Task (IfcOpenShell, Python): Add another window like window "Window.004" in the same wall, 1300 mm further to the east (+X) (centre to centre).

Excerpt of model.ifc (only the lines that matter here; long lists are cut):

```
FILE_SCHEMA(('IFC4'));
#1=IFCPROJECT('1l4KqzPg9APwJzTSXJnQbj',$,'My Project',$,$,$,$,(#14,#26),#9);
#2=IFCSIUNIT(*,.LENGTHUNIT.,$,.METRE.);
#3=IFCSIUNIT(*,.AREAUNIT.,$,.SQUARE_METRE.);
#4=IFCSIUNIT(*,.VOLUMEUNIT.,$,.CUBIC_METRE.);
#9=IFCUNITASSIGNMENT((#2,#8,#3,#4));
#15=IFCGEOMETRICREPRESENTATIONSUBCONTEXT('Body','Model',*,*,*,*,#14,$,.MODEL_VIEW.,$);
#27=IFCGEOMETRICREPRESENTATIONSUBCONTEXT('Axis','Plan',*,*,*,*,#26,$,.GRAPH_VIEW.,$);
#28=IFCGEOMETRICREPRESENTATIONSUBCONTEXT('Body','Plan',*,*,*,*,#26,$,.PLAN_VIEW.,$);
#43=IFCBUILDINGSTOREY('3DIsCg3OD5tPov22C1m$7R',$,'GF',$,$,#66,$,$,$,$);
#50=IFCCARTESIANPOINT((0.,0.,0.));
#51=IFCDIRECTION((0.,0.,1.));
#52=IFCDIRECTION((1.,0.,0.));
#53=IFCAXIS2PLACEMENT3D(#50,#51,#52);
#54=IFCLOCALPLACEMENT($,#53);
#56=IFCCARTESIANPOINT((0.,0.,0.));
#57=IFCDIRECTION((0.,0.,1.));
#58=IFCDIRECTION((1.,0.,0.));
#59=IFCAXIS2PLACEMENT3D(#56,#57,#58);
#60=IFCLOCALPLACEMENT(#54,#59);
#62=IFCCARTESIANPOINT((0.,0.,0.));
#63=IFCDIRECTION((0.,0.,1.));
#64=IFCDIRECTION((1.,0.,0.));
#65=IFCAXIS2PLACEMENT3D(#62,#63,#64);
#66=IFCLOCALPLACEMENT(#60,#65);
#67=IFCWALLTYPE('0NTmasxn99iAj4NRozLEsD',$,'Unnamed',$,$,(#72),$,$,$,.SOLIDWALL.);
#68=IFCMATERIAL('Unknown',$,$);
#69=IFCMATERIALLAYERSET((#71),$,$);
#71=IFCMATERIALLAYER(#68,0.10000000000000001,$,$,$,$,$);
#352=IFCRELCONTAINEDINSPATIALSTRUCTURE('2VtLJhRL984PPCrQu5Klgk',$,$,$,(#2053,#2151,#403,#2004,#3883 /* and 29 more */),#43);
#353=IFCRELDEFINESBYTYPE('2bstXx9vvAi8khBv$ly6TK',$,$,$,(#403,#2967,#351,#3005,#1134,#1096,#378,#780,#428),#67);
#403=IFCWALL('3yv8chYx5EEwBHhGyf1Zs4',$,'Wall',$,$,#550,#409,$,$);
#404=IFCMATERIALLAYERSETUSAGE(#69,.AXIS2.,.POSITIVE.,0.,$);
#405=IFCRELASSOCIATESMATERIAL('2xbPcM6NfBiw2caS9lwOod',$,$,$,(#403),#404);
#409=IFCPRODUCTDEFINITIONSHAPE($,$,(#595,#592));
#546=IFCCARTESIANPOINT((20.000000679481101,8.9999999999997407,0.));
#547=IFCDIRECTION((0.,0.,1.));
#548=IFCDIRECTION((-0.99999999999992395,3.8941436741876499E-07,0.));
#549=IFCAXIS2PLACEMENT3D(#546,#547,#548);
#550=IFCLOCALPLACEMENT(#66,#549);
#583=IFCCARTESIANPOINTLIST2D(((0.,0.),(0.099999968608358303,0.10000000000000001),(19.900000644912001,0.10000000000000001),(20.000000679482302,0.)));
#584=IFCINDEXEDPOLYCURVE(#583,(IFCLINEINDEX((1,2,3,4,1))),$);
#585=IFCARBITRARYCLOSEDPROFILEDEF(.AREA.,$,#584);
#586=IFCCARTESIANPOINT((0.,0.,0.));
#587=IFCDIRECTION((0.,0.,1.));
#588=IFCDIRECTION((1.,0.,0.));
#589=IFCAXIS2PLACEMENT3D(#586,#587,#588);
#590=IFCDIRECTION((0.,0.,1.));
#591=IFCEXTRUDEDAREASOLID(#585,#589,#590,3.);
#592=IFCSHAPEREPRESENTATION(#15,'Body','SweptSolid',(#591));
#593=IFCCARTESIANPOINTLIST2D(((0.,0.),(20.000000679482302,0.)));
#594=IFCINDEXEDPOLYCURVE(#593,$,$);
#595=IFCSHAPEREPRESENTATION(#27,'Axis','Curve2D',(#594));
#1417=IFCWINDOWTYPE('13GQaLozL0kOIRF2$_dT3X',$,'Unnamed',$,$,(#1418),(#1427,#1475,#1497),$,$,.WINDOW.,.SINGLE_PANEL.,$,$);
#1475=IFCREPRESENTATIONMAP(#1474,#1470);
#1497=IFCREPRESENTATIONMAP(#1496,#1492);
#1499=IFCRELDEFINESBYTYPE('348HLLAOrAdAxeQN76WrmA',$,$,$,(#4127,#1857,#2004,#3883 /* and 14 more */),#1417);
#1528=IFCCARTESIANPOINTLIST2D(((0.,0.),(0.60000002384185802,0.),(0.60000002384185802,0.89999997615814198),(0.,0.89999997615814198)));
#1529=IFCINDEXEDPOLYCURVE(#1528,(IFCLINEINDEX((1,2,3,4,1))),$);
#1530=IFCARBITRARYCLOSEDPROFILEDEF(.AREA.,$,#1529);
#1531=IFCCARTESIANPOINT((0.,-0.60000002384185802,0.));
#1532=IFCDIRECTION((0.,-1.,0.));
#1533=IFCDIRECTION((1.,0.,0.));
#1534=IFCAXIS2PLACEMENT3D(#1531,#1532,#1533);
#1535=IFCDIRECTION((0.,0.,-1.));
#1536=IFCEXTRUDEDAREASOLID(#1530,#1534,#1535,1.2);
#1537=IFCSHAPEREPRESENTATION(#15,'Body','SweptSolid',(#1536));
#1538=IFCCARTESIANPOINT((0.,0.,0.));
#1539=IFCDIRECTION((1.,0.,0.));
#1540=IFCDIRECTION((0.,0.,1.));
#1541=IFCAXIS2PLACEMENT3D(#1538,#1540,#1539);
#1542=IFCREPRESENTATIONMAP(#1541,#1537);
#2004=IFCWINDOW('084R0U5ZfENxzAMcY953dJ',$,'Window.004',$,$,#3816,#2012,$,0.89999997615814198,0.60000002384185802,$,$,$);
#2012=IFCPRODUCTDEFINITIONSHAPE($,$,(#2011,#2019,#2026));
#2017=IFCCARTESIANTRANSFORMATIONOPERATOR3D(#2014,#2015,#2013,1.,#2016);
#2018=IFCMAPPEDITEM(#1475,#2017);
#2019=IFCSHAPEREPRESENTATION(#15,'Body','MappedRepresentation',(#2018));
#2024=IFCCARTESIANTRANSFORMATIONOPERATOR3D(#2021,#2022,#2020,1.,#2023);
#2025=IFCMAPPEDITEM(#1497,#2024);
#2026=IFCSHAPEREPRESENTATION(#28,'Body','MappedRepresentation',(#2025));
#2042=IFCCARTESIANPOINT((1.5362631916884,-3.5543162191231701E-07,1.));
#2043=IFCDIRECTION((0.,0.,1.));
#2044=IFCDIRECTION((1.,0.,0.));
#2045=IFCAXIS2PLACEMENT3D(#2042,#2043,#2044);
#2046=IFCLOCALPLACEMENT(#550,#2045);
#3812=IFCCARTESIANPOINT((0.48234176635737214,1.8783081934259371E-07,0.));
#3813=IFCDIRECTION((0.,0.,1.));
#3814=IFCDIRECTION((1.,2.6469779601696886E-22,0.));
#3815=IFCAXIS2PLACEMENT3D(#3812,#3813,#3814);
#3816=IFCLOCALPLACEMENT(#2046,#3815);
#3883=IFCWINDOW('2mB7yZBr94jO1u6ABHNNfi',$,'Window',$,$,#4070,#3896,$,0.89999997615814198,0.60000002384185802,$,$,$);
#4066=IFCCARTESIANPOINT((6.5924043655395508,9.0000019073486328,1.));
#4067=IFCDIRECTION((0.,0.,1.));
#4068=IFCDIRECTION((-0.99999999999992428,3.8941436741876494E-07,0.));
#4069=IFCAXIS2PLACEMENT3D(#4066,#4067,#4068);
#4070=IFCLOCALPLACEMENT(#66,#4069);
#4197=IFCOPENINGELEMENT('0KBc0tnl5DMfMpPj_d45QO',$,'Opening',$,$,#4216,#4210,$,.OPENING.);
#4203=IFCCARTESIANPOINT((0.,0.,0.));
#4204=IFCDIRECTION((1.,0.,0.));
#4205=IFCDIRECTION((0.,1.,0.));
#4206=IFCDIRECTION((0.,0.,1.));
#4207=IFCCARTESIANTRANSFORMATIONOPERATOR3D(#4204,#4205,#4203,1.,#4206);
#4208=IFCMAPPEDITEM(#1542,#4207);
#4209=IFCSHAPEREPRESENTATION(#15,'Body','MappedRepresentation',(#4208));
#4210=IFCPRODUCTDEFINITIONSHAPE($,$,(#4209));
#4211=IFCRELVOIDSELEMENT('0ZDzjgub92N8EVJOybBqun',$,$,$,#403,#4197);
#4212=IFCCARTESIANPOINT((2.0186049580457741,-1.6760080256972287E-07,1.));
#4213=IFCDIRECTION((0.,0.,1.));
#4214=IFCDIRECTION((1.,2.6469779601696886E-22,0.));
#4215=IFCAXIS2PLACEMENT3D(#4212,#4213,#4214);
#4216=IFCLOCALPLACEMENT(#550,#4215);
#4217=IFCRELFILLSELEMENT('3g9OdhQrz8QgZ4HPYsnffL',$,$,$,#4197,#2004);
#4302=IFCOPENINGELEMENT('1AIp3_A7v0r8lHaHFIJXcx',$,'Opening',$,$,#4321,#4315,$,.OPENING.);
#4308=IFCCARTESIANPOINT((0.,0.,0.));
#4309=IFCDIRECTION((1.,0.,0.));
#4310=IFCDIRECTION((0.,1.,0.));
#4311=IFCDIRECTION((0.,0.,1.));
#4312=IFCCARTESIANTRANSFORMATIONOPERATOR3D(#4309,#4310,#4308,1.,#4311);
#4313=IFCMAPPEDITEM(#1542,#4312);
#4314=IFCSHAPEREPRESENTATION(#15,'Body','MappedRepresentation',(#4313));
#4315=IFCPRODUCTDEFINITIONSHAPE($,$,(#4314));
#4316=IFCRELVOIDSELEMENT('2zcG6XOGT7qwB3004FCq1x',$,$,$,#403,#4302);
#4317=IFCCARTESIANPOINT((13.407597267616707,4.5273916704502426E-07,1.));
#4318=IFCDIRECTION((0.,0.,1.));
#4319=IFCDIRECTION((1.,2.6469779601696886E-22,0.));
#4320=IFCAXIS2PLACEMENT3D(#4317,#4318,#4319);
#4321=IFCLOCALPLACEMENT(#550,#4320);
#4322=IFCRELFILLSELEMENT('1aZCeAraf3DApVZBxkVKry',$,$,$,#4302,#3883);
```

```python
import ifcopenshell
import ifcopenshell.api.feature
import ifcopenshell.api.geometry
import ifcopenshell.api.root
import ifcopenshell.geom
import ifcopenshell.util.element
import ifcopenshell.util.placement
import ifcopenshell.util.shape
import ifcopenshell.util.unit

model = ifcopenshell.open("model.ifc")
unit_scale = ifcopenshell.util.unit.calculate_unit_scale(model)
settings = ifcopenshell.geom.settings()


def volume(element):
    """Net volume in cubic metres, openings subtracted."""
    shape = ifcopenshell.geom.create_shape(settings, element)
    return ifcopenshell.util.shape.get_volume(shape.geometry)


window = model.by_id(2004)
opening = window.FillsVoids[0].RelatingOpeningElement
wall = opening.VoidsElements[0].RelatingBuildingElement
before = volume(wall)
shift = ifcopenshell.util.placement.get_local_placement(wall.ObjectPlacement)[:3, 0] * -1.3 / unit_scale

# copy_class copies the void relationship, type, container and properties, but no geometry.
new_opening = ifcopenshell.api.root.copy_class(model, product=opening)
new_opening.Representation = ifcopenshell.util.element.copy_deep(
    model, opening.Representation, exclude=["IfcGeometricRepresentationContext", "IfcRepresentationMap"]
)
new_window = ifcopenshell.api.root.copy_class(model, product=window)
new_window.Representation = ifcopenshell.util.element.copy_deep(
    model, window.Representation, exclude=["IfcGeometricRepresentationContext", "IfcRepresentationMap"]
)
ifcopenshell.api.feature.add_filling(model, opening=new_opening, element=new_window)

for old, new in ((opening, new_opening), (window, new_window)):
    matrix = ifcopenshell.util.placement.get_local_placement(old.ObjectPlacement)
    matrix[:3, 3] += shift
    ifcopenshell.api.geometry.edit_object_placement(model, product=new, matrix=matrix, is_si=False)

after = volume(wall)

print(f"wall volume {before:.3f} -> {after:.3f} m3")

model.write("model_v2.ifc")
```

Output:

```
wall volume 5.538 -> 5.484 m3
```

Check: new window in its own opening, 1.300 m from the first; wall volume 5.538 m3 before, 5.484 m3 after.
